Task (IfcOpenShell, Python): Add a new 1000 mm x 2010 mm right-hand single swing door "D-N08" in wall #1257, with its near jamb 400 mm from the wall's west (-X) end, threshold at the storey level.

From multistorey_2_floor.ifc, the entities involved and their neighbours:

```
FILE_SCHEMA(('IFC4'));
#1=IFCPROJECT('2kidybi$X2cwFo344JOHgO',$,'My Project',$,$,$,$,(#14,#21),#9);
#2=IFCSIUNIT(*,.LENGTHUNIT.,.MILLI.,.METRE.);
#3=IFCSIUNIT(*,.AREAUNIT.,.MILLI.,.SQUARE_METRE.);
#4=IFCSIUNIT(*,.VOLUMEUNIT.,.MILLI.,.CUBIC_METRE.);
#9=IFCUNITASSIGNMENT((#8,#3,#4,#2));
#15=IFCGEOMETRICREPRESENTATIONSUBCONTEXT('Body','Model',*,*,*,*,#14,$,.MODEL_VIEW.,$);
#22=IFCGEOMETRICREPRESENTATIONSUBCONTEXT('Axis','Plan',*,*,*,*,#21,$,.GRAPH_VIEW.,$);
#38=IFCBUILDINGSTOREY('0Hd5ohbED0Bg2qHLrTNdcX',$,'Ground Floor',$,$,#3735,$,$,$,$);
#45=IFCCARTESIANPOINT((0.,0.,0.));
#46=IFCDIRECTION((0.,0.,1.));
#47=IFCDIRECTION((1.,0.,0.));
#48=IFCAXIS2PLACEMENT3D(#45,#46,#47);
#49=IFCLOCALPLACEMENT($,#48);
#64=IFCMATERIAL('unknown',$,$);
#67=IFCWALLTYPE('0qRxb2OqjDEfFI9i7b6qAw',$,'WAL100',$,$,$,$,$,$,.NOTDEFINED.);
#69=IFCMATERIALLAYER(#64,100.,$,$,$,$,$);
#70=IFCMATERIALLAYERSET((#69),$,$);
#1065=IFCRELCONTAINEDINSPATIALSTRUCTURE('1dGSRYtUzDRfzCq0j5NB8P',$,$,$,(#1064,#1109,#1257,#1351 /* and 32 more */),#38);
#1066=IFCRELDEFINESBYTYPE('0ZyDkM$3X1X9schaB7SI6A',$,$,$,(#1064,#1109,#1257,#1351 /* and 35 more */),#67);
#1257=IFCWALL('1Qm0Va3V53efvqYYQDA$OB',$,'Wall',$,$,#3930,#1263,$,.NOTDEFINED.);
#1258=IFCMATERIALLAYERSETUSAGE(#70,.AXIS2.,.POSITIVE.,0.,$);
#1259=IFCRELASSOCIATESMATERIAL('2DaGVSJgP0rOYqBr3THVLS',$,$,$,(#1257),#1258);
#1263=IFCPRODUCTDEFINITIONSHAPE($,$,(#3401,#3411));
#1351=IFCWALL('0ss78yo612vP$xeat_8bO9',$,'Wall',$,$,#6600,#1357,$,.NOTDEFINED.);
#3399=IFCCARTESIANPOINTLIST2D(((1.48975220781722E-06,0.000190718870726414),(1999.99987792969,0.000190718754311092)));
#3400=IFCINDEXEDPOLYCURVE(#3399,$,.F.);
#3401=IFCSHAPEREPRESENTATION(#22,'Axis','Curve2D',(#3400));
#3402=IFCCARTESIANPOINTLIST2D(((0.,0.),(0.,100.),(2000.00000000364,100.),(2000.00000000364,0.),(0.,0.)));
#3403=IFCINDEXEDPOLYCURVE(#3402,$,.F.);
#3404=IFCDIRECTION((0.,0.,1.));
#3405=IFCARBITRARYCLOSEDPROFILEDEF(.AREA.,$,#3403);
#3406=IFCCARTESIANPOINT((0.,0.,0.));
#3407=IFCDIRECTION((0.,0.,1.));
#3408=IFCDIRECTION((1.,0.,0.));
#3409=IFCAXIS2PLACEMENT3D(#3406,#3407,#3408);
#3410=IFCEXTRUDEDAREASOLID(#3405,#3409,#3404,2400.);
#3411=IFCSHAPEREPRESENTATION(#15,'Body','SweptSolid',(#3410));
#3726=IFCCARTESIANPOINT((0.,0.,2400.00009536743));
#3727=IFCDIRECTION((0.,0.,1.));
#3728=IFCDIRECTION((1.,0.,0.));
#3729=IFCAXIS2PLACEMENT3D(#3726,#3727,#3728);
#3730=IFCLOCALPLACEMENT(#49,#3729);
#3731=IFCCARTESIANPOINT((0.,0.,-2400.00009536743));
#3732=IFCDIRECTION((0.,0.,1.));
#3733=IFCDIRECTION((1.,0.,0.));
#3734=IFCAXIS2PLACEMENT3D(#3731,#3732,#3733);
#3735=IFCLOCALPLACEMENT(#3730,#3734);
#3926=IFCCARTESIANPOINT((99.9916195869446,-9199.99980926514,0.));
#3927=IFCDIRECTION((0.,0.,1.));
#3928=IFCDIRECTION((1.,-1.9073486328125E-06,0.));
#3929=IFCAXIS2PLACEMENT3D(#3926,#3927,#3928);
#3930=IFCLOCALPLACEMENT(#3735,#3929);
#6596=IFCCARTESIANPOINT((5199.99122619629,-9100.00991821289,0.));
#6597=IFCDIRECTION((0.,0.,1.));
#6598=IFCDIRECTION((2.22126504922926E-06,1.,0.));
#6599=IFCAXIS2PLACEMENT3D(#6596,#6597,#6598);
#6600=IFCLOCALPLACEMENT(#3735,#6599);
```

```python
import numpy as np
import ifcopenshell
import ifcopenshell.api.feature
import ifcopenshell.api.geometry
import ifcopenshell.api.root
import ifcopenshell.api.spatial
import ifcopenshell.geom
import ifcopenshell.util.element
import ifcopenshell.util.placement
import ifcopenshell.util.representation
import ifcopenshell.util.shape
import ifcopenshell.util.unit

model = ifcopenshell.open("multistorey_2_floor.ifc")
unit_scale = ifcopenshell.util.unit.calculate_unit_scale(model)
settings = ifcopenshell.geom.settings()


def volume(element):
    """Net volume in cubic metres, openings subtracted."""
    shape = ifcopenshell.geom.create_shape(settings, element)
    return ifcopenshell.util.shape.get_volume(shape.geometry)


wall = model.by_guid("1Qm0Va3V53efvqYYQDA$OB")
storey = ifcopenshell.util.element.get_container(wall, ifc_class="IfcBuildingStorey")
context = ifcopenshell.util.representation.get_context(model, "Model", "Body", "MODEL_VIEW")
before = volume(wall)

width, height, from_end, sill = 1, 2.01, 0.4, 0.0  # metres

# The wall runs along its own X axis, and the end named is its -X end.
wall_shape = ifcopenshell.geom.create_shape(settings, wall)
x, y, z = ifcopenshell.util.shape.get_vertices(wall_shape.geometry).T
start = x.min() + from_end
face, thickness = float(y.min()), float(y.max() - y.min())
wall_matrix = ifcopenshell.util.placement.get_local_placement(wall.ObjectPlacement)
level = ifcopenshell.util.placement.get_local_placement(storey.ObjectPlacement)[2, 3]


def in_wall(x, y):
    """Placement at x, y metres in the wall's axes, at sill height."""
    matrix = wall_matrix.copy()
    matrix[:, 3] = wall_matrix @ np.array([x / unit_scale, y / unit_scale, 0.0, 1.0])
    matrix[2, 3] = level + sill / unit_scale
    return matrix


# Opening: a box that overshoots both wall faces by 50 mm.
opening = ifcopenshell.api.root.create_entity(model, ifc_class="IfcOpeningElement", predefined_type="OPENING")
box = ifcopenshell.api.geometry.add_wall_representation(
    model, context=context, length=width, height=height, thickness=thickness + 0.1
)
ifcopenshell.api.geometry.assign_representation(model, product=opening, representation=box)
ifcopenshell.api.geometry.edit_object_placement(model, product=opening, matrix=in_wall(start, face - 0.05), is_si=False)
ifcopenshell.api.feature.add_feature(model, feature=opening, element=wall)

door = ifcopenshell.api.root.create_entity(model, ifc_class="IfcDoor", name="D-N08", predefined_type="DOOR")
door.OverallWidth, door.OverallHeight = width / unit_scale, height / unit_scale
door.OperationType = "SINGLE_SWING_RIGHT"
body = ifcopenshell.api.geometry.add_door_representation(
    model,
    context=context,
    overall_width=door.OverallWidth,
    overall_height=door.OverallHeight,
    operation_type="SINGLE_SWING_RIGHT",
    lining_properties={"LiningDepth": thickness / unit_scale, "ThresholdDepth": thickness / unit_scale},
)
ifcopenshell.api.geometry.assign_representation(model, product=door, representation=body)
ifcopenshell.api.spatial.assign_container(model, products=[door], relating_structure=storey)
ifcopenshell.api.feature.add_filling(model, opening=opening, element=door)

# The lining spans the wall, so the door starts at the wall face.
ifcopenshell.api.geometry.edit_object_placement(model, product=door, matrix=in_wall(start, face), is_si=False)

after = volume(wall)

print(f"wall volume {before:.3f} -> {after:.3f} m3")

model.write("multistorey_2_floor_rev.ifc")
```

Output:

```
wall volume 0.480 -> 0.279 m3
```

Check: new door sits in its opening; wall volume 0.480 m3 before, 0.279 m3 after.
